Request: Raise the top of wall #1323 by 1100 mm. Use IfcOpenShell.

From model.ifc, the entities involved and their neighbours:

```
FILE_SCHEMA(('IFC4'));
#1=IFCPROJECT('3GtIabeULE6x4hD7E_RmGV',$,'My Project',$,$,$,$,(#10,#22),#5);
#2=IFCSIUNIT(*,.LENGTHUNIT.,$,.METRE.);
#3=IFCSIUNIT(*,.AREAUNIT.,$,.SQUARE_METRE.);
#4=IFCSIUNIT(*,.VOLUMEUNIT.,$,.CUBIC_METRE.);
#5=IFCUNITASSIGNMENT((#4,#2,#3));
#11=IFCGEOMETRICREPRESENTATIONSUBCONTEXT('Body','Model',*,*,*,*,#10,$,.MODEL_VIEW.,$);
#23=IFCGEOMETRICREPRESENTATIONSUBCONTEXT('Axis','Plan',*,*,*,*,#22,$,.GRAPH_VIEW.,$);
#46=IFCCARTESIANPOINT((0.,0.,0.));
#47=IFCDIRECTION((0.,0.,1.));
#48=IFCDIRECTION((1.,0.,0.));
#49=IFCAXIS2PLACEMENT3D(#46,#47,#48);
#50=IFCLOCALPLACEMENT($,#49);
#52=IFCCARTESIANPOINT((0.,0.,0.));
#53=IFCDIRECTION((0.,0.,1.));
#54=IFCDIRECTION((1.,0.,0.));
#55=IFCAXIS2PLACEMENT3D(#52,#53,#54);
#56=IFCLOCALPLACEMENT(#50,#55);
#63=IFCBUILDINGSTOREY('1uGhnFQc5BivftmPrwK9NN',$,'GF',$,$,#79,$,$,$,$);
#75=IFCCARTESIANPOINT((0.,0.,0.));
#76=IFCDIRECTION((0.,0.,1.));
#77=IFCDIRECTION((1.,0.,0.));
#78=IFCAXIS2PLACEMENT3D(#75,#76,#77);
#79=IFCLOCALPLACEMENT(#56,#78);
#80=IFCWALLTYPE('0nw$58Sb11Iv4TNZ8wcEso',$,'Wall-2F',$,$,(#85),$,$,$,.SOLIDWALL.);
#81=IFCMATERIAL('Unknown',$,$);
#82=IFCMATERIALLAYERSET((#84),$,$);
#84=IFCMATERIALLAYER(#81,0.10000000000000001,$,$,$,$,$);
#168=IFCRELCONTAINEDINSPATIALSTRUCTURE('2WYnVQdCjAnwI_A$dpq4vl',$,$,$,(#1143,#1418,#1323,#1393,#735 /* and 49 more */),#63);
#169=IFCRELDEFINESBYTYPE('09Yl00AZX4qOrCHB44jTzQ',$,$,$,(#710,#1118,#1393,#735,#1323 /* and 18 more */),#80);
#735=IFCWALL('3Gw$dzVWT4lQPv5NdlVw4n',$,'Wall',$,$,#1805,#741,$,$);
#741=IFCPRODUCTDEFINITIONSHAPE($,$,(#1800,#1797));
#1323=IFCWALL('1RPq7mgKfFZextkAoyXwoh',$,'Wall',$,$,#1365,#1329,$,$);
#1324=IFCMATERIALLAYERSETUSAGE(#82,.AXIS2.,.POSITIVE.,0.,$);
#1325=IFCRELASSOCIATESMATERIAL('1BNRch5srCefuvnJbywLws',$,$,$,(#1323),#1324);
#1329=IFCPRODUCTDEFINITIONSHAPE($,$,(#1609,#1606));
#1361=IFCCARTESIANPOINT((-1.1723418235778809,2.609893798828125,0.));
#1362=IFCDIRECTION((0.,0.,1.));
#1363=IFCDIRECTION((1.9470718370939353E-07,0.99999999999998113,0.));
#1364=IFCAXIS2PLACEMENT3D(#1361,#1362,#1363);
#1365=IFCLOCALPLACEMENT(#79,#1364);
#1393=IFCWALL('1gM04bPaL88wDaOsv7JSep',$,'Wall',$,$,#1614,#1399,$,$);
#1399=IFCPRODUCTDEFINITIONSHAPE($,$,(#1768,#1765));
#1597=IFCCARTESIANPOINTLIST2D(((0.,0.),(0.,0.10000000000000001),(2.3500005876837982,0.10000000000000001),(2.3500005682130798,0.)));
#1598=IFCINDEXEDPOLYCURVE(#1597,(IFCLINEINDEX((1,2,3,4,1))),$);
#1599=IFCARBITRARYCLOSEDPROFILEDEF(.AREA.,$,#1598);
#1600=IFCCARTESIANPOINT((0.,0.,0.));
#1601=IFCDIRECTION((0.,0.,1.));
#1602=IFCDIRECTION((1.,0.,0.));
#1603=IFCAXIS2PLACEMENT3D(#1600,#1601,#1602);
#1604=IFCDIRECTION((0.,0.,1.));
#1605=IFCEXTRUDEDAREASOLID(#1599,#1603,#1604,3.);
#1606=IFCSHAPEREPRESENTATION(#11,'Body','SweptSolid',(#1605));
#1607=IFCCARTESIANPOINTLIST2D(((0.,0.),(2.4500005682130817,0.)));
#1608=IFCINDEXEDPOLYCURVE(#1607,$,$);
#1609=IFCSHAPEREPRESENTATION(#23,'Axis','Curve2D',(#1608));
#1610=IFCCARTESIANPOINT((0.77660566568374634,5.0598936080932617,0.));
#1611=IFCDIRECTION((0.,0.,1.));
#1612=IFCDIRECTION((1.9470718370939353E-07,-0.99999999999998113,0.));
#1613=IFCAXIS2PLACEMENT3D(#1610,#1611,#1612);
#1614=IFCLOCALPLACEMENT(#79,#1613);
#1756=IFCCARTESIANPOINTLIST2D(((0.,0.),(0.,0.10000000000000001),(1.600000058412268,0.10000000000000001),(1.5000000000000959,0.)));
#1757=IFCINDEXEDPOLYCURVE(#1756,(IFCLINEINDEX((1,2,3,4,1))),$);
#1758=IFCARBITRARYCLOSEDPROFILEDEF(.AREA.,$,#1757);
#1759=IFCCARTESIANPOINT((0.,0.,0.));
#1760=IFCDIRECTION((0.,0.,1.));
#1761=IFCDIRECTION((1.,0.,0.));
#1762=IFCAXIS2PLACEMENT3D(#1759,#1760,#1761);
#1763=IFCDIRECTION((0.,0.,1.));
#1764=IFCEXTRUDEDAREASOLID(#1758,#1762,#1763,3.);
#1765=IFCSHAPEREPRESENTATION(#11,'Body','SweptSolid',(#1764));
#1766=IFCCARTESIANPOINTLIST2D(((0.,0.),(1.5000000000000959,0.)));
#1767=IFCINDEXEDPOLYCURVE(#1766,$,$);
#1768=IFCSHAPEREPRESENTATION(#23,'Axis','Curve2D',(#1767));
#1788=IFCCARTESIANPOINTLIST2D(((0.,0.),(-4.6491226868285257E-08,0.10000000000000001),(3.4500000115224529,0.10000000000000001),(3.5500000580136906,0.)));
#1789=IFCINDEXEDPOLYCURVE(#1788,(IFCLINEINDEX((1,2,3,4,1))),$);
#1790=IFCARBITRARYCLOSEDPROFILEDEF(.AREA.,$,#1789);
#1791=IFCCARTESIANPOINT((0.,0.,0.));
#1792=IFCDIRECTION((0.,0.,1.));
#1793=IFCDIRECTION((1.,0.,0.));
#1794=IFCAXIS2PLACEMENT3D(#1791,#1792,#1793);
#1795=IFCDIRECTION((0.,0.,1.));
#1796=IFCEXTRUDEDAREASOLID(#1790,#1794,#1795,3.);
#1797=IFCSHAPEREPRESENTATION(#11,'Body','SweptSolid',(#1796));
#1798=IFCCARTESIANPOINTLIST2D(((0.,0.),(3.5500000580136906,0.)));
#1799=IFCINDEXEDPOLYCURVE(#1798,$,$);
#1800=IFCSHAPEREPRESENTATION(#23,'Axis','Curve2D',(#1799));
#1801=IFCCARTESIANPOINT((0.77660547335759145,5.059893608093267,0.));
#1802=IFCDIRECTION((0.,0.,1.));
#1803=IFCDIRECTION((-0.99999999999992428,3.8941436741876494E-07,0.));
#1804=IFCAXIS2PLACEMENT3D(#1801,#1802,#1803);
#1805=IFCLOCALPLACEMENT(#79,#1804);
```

```python
import ifcopenshell
import ifcopenshell.geom
import ifcopenshell.util.representation
import ifcopenshell.util.shape
import ifcopenshell.util.unit

model = ifcopenshell.open("model.ifc")
unit_scale = ifcopenshell.util.unit.calculate_unit_scale(model)
settings = ifcopenshell.geom.settings()


def volume(element):
    """Net volume in cubic metres, openings subtracted."""
    shape = ifcopenshell.geom.create_shape(settings, element)
    return ifcopenshell.util.shape.get_volume(shape.geometry)


wall = model.by_guid("1RPq7mgKfFZextkAoyXwoh")
before = volume(wall)

body = ifcopenshell.util.representation.get_representation(wall, "Model", "Body")
solid = body.Items[0]
old_height = solid.Depth
solid.Depth += 1.1 / unit_scale
after = volume(wall)

print(f"height {old_height:g} -> {solid.Depth:g}, volume {before:.3f} -> {after:.3f} m3")

model.write("model_updated.ifc")
```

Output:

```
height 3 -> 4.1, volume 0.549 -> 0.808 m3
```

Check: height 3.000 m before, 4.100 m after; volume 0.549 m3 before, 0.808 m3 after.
